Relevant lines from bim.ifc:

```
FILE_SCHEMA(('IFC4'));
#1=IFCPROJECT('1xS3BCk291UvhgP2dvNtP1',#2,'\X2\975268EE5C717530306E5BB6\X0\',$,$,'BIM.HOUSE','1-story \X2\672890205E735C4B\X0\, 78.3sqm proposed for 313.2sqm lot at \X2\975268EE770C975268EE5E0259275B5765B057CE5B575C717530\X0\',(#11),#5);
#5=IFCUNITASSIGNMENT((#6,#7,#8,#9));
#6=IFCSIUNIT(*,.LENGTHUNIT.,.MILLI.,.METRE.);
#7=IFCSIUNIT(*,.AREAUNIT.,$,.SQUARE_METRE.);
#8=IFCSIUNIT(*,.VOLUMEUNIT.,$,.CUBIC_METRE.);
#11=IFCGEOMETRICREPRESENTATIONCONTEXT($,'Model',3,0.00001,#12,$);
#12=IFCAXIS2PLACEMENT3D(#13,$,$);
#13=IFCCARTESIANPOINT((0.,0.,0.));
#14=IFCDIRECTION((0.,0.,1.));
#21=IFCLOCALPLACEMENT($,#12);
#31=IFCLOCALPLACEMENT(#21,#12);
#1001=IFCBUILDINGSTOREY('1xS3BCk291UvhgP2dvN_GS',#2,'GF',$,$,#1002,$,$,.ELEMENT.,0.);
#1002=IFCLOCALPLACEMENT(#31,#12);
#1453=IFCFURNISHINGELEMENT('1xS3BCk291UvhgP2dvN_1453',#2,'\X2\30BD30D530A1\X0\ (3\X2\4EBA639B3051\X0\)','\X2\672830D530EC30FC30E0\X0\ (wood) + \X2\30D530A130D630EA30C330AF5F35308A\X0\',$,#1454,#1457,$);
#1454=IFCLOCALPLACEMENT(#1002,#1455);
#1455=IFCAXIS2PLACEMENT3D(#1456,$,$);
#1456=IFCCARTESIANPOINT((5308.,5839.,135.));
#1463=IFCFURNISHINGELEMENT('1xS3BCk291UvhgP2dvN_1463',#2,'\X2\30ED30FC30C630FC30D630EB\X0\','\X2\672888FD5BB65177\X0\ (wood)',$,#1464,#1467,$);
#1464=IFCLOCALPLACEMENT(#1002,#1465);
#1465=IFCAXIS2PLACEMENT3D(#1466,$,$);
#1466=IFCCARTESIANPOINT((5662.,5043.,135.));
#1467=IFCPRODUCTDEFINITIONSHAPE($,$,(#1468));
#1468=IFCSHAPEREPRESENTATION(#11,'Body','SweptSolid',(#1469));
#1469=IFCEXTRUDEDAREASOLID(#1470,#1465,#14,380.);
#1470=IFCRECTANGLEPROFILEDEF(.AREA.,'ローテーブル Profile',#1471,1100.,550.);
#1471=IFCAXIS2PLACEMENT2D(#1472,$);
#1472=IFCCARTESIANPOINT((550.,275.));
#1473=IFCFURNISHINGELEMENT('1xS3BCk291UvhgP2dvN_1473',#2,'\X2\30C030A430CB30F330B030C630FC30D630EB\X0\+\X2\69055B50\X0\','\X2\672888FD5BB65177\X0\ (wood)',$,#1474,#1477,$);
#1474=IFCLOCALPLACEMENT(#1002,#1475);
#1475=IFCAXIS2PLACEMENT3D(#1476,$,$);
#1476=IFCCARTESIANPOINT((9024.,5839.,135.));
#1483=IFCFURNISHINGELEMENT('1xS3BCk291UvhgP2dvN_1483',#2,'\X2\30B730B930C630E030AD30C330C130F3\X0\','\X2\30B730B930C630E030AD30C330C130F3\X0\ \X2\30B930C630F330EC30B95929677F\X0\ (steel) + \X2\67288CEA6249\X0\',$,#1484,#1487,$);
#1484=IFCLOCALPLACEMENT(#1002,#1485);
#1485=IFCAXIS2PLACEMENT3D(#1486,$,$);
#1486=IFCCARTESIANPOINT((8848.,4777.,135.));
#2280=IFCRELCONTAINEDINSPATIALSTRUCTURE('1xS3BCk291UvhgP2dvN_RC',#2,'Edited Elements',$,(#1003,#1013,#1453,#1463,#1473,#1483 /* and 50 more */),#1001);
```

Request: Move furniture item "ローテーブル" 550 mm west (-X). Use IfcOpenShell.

```python
import ifcopenshell
import ifcopenshell.api.geometry
import ifcopenshell.util.placement
import ifcopenshell.util.unit

model = ifcopenshell.open("bim.ifc")
unit_scale = ifcopenshell.util.unit.calculate_unit_scale(model)

item = model.by_id(1463)
matrix = ifcopenshell.util.placement.get_local_placement(item.ObjectPlacement)
matrix[0, 3] -= 0.55 / unit_scale
ifcopenshell.api.geometry.edit_object_placement(model, product=item, matrix=matrix, is_si=False)

print(ifcopenshell.util.placement.get_local_placement(item.ObjectPlacement).round(3) + 0.0)

model.write("bim_v2.ifc")
```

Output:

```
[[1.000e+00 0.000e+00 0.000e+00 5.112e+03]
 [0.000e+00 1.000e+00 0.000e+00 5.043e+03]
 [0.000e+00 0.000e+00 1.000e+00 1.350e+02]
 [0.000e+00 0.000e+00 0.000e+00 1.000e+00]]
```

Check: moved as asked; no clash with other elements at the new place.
